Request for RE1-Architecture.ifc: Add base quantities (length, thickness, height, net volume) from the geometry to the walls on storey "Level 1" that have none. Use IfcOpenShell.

First a look at what the model holds.

```python
import ifcopenshell
import ifcopenshell.util.element
import ifcopenshell.util.unit

model = ifcopenshell.open("RE1-Architecture.ifc")
print(model.schema)
for unit_type in ("LENGTHUNIT", "AREAUNIT", "VOLUMEUNIT"):
    print(unit_type, ifcopenshell.util.unit.calculate_unit_scale(model, unit_type))
storey = next(s for s in model.by_type("IfcBuildingStorey") if s.Name == "Level 1")
walls = [e for e in ifcopenshell.util.element.get_decomposition(storey) if e.is_a("IfcWall")]
for e in sorted(walls, key=lambda e: e.id()):
    print(e.id(), e.is_a(), e.Name, list(ifcopenshell.util.element.get_psets(e, qtos_only=True)), sep=" | ")
```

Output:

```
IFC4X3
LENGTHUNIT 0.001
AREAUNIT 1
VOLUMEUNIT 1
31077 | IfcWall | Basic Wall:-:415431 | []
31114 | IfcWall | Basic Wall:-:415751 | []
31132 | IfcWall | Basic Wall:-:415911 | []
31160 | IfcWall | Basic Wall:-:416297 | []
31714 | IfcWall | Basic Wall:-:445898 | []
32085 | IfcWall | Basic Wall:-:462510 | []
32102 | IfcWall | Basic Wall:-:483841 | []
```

```python
import ifcopenshell
import ifcopenshell.api.pset
import ifcopenshell.geom
import ifcopenshell.util.element
import ifcopenshell.util.shape
import ifcopenshell.util.unit

model = ifcopenshell.open("RE1-Architecture.ifc")
unit_scale = ifcopenshell.util.unit.calculate_unit_scale(model)
volume_scale = ifcopenshell.util.unit.calculate_unit_scale(model, "VOLUMEUNIT")
settings = ifcopenshell.geom.settings()

storey = next(s for s in model.by_type("IfcBuildingStorey") if s.Name == "Level 1")
walls = [e for e in ifcopenshell.util.element.get_decomposition(storey) if e.is_a("IfcWall")]

for e in sorted(walls, key=lambda e: e.id()):
    if ifcopenshell.util.element.get_psets(e, qtos_only=True, should_inherit=False):
        continue
    # Geometry comes back in metres, in the element's own axes.
    shape = ifcopenshell.geom.create_shape(settings, e)
    values = {
        "Length": ifcopenshell.util.shape.get_x(shape.geometry) / unit_scale,
        "Width": ifcopenshell.util.shape.get_y(shape.geometry) / unit_scale,
        "Height": ifcopenshell.util.shape.get_z(shape.geometry) / unit_scale,
        "NetVolume": ifcopenshell.util.shape.get_volume(shape.geometry) / volume_scale,
    }
    qto = ifcopenshell.api.pset.add_qto(model, product=e, name="Qto_WallBaseQuantities")
    ifcopenshell.api.pset.edit_qto(model, qto=qto, properties=values)
    print(e.id(), {k: round(v, 3) for k, v in values.items()})

model.write("RE1-Architecture_edited.ifc")
```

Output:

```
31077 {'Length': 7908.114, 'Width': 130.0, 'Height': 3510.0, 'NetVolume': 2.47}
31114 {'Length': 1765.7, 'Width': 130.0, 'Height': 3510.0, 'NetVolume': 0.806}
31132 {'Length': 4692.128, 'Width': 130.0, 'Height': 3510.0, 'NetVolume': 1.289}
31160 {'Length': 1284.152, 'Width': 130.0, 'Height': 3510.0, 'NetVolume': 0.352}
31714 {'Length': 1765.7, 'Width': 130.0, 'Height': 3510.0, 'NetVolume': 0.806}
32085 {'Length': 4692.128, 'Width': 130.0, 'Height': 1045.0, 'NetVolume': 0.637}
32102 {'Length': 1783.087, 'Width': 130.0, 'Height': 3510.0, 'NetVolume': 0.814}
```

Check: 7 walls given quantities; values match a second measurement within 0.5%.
